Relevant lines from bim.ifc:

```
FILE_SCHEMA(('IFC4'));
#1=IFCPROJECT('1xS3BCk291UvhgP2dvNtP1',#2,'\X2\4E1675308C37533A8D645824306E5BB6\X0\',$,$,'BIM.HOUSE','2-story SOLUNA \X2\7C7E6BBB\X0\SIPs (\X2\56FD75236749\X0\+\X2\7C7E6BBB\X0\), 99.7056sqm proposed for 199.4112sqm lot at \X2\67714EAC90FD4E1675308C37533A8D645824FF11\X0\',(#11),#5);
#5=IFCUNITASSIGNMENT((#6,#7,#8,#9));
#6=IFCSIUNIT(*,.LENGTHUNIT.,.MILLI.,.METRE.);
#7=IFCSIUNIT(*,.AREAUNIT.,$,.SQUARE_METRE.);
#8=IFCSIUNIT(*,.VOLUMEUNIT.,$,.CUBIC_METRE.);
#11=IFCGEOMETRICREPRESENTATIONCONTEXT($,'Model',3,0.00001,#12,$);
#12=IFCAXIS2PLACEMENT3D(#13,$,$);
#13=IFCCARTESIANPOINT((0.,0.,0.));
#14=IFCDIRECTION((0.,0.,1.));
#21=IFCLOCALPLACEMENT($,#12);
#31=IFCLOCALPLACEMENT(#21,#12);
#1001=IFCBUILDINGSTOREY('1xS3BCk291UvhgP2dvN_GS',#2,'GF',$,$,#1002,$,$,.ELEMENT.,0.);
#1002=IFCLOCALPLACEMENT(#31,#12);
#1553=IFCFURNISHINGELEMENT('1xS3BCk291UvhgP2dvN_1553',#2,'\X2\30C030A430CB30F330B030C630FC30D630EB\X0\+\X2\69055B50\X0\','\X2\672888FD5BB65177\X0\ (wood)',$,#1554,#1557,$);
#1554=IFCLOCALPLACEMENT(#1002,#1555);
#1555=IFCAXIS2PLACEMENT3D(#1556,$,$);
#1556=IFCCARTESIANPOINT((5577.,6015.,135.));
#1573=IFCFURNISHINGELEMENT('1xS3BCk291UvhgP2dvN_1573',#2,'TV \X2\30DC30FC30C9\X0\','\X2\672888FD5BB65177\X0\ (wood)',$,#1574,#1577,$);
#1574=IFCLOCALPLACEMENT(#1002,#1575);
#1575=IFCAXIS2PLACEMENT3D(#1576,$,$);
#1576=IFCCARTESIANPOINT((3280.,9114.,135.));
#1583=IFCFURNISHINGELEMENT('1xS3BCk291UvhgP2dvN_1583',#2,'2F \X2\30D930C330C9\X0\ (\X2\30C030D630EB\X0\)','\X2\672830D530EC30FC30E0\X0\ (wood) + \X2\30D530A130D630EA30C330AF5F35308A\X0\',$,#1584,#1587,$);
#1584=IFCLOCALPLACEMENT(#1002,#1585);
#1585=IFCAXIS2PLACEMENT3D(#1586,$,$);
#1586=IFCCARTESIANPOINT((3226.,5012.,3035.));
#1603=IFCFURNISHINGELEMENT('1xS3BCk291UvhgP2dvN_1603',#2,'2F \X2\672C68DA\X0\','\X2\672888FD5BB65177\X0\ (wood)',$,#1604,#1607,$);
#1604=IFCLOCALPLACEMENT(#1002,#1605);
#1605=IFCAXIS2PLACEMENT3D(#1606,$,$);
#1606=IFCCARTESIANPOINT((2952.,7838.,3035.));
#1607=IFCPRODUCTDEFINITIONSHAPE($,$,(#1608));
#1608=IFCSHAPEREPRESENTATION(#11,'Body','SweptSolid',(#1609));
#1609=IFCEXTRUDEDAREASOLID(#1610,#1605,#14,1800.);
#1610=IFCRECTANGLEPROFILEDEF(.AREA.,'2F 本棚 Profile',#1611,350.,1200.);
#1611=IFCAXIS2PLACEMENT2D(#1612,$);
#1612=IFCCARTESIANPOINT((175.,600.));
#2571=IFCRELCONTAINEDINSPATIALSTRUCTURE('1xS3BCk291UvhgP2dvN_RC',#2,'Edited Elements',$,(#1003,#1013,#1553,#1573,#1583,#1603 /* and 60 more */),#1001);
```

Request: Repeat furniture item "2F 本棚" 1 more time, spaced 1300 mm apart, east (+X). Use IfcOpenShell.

```python
import numpy as np
import ifcopenshell
import ifcopenshell.api.geometry
import ifcopenshell.api.root
import ifcopenshell.util.element
import ifcopenshell.util.placement
import ifcopenshell.util.unit

model = ifcopenshell.open("bim.ifc")
unit_scale = ifcopenshell.util.unit.calculate_unit_scale(model)


def reuse_history(source, copy):
    """copy_class also copies each property set's owner history, people and application; keep the originals."""
    for rel in copy.IsDefinedBy:
        if rel.is_a("IfcRelDefinesByProperties") and (history := rel.RelatingPropertyDefinition.OwnerHistory):
            rel.RelatingPropertyDefinition.OwnerHistory = source.OwnerHistory
            ifcopenshell.util.element.remove_deep2(model, history)


source = model.by_guid("1xS3BCk291UvhgP2dvN_1603")
base = ifcopenshell.util.placement.get_local_placement(source.ObjectPlacement)
step = np.array([1.0, 0.0, 0.0]) * 1.3 / unit_scale

for i in range(1, 2):
    copy = ifcopenshell.api.root.copy_class(model, product=source)
    copy.Representation = ifcopenshell.util.element.copy_deep(
        model, source.Representation, exclude=["IfcGeometricRepresentationContext", "IfcRepresentationMap"]
    )
    reuse_history(source, copy)
    matrix = base.copy()
    matrix[:3, 3] += i * step
    print("added at", matrix[:3, 3].round(3) + 0.0)
    ifcopenshell.api.geometry.edit_object_placement(model, product=copy, matrix=matrix, is_si=False)

model.write("bim_rev.ifc")
```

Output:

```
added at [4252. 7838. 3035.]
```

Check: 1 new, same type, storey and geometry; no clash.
